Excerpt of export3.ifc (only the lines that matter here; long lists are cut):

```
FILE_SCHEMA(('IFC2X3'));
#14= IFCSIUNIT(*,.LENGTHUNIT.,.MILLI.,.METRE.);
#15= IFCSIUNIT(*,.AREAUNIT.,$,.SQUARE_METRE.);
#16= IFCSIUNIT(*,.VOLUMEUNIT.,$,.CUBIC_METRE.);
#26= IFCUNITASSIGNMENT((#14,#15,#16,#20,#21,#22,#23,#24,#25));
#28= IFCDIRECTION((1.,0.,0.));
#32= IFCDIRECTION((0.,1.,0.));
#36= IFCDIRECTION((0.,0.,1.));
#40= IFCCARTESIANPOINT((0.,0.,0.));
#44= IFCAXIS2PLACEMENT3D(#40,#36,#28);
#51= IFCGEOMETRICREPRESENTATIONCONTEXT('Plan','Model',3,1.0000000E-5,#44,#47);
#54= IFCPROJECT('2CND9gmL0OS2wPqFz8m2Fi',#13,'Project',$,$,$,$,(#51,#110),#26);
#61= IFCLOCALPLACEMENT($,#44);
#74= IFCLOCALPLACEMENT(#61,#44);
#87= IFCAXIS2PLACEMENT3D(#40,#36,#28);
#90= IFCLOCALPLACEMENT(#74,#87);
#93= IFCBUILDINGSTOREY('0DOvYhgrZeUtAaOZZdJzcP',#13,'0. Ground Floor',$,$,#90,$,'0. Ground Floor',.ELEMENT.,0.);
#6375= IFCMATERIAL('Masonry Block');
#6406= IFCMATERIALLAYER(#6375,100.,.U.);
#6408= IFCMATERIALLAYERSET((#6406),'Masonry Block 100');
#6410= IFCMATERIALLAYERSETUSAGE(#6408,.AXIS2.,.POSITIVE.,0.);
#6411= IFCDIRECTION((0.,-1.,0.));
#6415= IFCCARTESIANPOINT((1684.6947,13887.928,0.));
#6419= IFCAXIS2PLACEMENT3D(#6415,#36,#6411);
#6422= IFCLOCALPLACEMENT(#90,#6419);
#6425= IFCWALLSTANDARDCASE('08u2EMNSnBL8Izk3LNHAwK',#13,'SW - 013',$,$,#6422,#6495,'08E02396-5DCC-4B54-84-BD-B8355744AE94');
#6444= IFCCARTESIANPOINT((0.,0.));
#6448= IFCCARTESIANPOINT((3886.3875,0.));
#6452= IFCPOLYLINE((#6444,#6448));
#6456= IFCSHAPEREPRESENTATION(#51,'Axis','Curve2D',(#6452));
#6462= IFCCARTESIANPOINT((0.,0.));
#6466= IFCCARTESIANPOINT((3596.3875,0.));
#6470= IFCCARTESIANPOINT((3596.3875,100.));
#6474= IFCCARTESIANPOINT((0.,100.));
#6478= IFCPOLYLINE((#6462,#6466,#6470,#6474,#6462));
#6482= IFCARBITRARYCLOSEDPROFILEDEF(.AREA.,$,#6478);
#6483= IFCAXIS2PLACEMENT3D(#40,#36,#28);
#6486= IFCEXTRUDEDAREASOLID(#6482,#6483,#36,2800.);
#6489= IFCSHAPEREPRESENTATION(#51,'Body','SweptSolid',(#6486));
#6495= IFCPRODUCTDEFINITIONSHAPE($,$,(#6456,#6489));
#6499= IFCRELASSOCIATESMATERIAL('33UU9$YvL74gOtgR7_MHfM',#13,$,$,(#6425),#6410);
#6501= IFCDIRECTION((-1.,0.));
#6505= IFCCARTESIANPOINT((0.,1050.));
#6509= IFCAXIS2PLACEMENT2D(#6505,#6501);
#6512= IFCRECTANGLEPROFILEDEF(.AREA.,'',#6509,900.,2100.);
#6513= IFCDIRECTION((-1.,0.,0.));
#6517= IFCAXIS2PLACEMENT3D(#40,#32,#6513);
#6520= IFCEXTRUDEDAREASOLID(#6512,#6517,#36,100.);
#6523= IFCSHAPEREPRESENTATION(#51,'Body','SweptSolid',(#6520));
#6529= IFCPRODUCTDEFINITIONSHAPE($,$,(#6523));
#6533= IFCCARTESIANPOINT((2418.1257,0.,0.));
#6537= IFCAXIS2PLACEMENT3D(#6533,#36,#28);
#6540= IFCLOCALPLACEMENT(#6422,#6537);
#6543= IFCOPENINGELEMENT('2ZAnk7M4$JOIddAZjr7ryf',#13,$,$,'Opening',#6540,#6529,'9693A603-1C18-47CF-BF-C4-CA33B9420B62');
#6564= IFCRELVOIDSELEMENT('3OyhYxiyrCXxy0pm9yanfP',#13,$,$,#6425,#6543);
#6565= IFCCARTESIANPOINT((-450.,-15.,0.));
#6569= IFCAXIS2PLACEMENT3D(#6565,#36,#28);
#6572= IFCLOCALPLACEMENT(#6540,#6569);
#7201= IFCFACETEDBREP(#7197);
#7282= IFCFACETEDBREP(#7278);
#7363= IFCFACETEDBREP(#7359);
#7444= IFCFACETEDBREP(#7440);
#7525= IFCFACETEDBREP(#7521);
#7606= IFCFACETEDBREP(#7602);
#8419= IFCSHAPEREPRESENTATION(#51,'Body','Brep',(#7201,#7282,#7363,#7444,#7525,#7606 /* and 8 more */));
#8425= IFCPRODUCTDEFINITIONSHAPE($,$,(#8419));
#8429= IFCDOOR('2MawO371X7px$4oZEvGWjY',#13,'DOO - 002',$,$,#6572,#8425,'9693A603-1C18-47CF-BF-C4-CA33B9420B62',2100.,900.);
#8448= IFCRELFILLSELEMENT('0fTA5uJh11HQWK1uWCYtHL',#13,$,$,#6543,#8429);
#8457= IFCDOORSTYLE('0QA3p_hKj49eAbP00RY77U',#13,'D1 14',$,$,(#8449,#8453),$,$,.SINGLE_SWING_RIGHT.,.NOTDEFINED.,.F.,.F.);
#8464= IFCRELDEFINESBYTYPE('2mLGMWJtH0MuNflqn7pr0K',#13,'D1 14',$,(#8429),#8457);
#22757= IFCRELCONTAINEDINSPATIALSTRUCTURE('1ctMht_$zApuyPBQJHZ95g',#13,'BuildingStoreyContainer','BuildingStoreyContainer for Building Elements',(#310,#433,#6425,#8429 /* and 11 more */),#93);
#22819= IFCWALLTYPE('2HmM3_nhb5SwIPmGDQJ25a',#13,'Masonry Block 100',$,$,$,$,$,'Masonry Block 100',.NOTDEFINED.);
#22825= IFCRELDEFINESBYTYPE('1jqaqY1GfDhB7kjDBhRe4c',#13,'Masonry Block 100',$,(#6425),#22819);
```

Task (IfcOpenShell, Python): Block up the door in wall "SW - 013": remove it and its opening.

```python
import ifcopenshell
import ifcopenshell.api.feature
import ifcopenshell.api.root
import ifcopenshell.geom
import ifcopenshell.util.shape

model = ifcopenshell.open("export3.ifc")
settings = ifcopenshell.geom.settings()


def volume(element):
    """Net volume in cubic metres, openings subtracted."""
    shape = ifcopenshell.geom.create_shape(settings, element)
    return ifcopenshell.util.shape.get_volume(shape.geometry)


door = model.by_guid("2MawO371X7px$4oZEvGWjY")
opening = door.FillsVoids[0].RelatingOpeningElement
wall = opening.VoidsElements[0].RelatingBuildingElement
before = volume(wall)

ifcopenshell.api.root.remove_product(model, product=door)
ifcopenshell.api.feature.remove_feature(model, feature=opening)

after = volume(wall)

print(f"wall volume {before:.3f} -> {after:.3f} m3")

model.write("export3-out.ifc")
```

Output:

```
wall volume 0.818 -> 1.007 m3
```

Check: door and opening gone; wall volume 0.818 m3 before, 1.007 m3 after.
